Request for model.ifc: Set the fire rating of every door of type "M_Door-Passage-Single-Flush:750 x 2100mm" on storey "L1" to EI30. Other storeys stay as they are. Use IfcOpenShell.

First a look at what the model holds.

```python
import ifcopenshell
import ifcopenshell.util.element

model = ifcopenshell.open("model.ifc")
print(model.schema)
storey = next(s for s in model.by_type("IfcBuildingStorey") if s.Name == "L1")
doors = [e for e in ifcopenshell.util.element.get_decomposition(storey) if e.is_a("IfcDoor")]
seen = {}
for e in doors:
    element_type = ifcopenshell.util.element.get_type(e)
    key = (element_type.Name if element_type != e and element_type else None, ifcopenshell.util.element.get_pset(e, "Pset_DoorCommon", "FireRating"))
    seen[key] = seen.get(key, 0) + 1
for (name, value), count in sorted(seen.items(), key=str):
    print(count, "x", name, "|", value)
```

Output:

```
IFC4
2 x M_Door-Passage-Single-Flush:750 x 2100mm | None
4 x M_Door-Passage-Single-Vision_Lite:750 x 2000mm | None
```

```python
import ifcopenshell
import ifcopenshell.api.pset
import ifcopenshell.util.element

model = ifcopenshell.open("model.ifc")

storey = next(s for s in model.by_type("IfcBuildingStorey") if s.Name == "L1")
doors = [e for e in ifcopenshell.util.element.get_decomposition(storey) if e.is_a("IfcDoor")]

count = 0
for e in doors:
    element_type = ifcopenshell.util.element.get_type(e)
    if element_type in (None, e) or element_type.Name != "M_Door-Passage-Single-Flush:750 x 2100mm":
        continue
    # add_pset returns the element's existing set when there is one.
    pset = ifcopenshell.api.pset.add_pset(model, product=e, name="Pset_DoorCommon")
    ifcopenshell.api.pset.edit_pset(model, pset=pset, properties={"FireRating": "EI30"})
    count += 1

print(count, "doors updated")

model.write("model_updated.ifc")
```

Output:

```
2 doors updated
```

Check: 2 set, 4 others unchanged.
